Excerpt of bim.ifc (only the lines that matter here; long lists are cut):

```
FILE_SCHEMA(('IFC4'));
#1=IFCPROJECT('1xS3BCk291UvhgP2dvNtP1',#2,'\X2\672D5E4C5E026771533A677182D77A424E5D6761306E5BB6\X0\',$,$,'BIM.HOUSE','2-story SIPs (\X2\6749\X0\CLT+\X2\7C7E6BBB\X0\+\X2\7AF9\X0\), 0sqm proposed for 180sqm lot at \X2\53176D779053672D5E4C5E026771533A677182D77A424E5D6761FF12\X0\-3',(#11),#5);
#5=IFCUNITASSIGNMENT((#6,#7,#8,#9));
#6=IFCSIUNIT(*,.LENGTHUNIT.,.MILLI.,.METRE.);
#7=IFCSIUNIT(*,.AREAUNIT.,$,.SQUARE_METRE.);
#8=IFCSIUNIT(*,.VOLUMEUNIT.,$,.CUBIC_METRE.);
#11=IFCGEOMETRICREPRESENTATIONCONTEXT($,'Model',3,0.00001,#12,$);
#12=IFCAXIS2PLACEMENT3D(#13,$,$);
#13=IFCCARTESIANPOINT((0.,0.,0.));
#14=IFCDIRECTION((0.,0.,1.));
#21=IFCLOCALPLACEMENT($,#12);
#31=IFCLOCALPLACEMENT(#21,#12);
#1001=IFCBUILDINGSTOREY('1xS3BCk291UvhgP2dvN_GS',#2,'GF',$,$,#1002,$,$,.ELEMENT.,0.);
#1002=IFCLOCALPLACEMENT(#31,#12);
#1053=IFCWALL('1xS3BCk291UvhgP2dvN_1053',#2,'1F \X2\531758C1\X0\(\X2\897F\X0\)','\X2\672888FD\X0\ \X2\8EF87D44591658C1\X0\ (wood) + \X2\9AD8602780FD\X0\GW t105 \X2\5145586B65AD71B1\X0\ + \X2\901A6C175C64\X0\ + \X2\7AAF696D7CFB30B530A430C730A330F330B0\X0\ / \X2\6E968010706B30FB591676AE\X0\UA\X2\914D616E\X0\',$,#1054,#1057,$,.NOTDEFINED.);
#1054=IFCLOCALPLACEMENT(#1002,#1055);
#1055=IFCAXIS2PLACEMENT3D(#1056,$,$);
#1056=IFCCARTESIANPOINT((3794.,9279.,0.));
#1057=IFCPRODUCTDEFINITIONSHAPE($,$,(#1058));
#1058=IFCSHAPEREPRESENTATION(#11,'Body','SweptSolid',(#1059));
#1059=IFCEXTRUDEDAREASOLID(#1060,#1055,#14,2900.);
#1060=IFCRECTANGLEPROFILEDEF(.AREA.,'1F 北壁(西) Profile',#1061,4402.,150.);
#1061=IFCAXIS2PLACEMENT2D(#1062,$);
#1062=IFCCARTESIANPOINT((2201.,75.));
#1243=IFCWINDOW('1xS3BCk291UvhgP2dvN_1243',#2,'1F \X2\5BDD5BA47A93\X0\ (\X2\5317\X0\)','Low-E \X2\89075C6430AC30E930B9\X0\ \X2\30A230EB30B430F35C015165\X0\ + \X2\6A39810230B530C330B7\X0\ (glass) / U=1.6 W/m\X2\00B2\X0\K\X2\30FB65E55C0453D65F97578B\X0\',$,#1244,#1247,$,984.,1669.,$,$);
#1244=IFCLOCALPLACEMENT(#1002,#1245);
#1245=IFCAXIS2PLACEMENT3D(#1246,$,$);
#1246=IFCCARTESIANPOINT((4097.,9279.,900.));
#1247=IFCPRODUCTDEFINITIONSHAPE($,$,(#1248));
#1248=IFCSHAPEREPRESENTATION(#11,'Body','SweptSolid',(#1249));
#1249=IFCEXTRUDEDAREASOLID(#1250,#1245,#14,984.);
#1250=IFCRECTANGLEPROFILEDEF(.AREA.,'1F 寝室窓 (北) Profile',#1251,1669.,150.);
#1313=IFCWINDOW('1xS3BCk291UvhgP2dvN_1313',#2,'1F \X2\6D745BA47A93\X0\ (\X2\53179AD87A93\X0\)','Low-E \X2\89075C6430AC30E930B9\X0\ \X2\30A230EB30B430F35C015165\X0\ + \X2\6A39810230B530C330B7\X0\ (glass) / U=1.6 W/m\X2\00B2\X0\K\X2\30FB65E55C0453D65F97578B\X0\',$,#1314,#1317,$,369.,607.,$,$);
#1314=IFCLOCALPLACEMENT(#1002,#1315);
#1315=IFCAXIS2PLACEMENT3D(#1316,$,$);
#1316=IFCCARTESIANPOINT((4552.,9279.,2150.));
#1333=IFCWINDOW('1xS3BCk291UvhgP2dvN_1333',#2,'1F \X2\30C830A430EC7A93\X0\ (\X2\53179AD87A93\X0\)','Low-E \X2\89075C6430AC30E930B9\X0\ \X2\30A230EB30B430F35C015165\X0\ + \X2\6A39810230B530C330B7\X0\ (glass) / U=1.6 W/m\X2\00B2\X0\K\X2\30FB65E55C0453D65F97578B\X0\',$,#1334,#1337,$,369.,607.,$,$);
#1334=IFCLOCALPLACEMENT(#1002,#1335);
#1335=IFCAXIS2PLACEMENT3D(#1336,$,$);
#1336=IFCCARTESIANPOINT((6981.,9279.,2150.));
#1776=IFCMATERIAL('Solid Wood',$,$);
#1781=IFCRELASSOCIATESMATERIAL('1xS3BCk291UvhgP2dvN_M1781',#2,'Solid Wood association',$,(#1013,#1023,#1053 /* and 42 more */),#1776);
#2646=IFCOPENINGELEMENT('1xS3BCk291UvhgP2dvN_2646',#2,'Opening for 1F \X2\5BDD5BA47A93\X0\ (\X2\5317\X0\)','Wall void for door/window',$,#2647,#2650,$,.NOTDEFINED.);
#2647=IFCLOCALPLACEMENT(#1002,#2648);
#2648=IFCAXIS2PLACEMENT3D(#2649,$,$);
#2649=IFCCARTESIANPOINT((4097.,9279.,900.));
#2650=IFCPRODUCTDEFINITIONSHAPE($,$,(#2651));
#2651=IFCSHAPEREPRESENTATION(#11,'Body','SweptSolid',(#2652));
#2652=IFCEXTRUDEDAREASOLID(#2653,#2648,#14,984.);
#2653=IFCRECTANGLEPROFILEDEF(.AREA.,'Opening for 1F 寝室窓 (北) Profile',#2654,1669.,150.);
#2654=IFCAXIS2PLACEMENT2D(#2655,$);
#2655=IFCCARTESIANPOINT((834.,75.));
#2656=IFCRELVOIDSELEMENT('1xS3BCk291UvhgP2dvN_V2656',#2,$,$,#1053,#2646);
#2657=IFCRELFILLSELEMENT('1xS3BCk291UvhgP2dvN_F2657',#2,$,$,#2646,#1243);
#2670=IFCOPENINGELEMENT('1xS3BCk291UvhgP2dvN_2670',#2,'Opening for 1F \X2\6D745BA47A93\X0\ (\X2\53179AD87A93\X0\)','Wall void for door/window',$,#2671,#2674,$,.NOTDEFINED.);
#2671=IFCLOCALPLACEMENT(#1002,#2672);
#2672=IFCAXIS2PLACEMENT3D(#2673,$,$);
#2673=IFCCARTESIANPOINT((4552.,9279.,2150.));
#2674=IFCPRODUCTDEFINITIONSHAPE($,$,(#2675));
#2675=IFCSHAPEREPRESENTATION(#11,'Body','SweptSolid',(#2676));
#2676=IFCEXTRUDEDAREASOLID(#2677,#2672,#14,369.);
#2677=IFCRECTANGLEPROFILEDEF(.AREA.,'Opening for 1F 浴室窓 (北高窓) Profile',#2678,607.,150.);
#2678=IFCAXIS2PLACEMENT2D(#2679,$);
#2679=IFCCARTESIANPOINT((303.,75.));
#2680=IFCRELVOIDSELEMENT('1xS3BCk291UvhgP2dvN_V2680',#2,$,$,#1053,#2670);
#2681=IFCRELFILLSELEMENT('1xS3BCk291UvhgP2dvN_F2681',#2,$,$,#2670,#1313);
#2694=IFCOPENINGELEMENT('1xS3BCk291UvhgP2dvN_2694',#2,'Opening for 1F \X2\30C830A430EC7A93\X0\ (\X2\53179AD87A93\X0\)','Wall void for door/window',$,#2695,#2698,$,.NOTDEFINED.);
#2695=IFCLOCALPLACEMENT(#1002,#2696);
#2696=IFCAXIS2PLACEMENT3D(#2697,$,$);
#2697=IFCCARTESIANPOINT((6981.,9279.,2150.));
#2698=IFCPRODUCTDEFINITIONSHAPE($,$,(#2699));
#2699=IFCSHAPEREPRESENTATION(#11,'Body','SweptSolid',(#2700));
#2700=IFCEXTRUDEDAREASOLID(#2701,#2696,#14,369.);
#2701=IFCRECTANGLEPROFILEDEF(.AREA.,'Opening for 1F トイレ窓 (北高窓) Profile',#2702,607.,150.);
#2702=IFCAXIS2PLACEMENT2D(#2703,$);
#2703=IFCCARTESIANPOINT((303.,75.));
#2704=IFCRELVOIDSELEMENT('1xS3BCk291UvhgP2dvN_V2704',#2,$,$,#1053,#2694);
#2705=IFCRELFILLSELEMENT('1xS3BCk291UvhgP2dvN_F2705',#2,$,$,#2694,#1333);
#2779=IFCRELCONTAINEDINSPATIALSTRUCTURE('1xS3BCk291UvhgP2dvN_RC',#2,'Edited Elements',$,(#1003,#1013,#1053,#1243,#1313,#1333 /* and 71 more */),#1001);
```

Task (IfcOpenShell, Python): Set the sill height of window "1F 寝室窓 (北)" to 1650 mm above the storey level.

```python
import numpy as np
import ifcopenshell
import ifcopenshell.api.geometry
import ifcopenshell.geom
import ifcopenshell.util.element
import ifcopenshell.util.placement
import ifcopenshell.util.shape
import ifcopenshell.util.unit

model = ifcopenshell.open("bim.ifc")
unit_scale = ifcopenshell.util.unit.calculate_unit_scale(model)

window = model.by_guid("1xS3BCk291UvhgP2dvN_1243")
opening = window.FillsVoids[0].RelatingOpeningElement
storey = ifcopenshell.util.element.get_container(window, ifc_class="IfcBuildingStorey")
level = ifcopenshell.util.placement.get_local_placement(storey.ObjectPlacement)[2, 3]

# The opening's origin need not be at the sill, so measure its lowest point.
shape = ifcopenshell.geom.create_shape(ifcopenshell.geom.settings(), opening)
bottom = ifcopenshell.util.shape.get_shape_bottom_elevation(shape, shape.geometry) / unit_scale
dz = level + 1650.0 - bottom

shift = np.array([0.0, 0.0, dz])
# The window is not placed relative to its opening, so move both.
for product in (opening, window):
    matrix = ifcopenshell.util.placement.get_local_placement(product.ObjectPlacement)
    matrix[:3, 3] += shift
    ifcopenshell.api.geometry.edit_object_placement(model, product=product, matrix=matrix, is_si=False)

print(f"moved by {dz * unit_scale:+.3f} m")

model.write("bim_updated.ifc")
```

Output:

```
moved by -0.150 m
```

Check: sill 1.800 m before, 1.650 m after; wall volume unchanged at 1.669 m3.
